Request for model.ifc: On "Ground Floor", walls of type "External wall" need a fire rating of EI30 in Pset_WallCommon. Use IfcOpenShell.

First a look at what the model holds.

```python
import ifcopenshell
import ifcopenshell.util.element

model = ifcopenshell.open("model.ifc")
print(model.schema)
storey = next(s for s in model.by_type("IfcBuildingStorey") if s.Name == "Ground Floor")
walls = [e for e in ifcopenshell.util.element.get_decomposition(storey) if e.is_a("IfcWall")]
seen = {}
for e in walls:
    element_type = ifcopenshell.util.element.get_type(e)
    key = (element_type.Name if element_type != e and element_type else None, ifcopenshell.util.element.get_pset(e, "Pset_WallCommon", "FireRating"))
    seen[key] = seen.get(key, 0) + 1
for (name, value), count in sorted(seen.items(), key=str):
    print(count, "x", name, "|", value)
```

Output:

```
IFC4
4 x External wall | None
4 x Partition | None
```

```python
import ifcopenshell
import ifcopenshell.api.pset
import ifcopenshell.util.element

model = ifcopenshell.open("model.ifc")

storey = next(s for s in model.by_type("IfcBuildingStorey") if s.Name == "Ground Floor")
walls = [e for e in ifcopenshell.util.element.get_decomposition(storey) if e.is_a("IfcWall")]

count = 0
for e in walls:
    element_type = ifcopenshell.util.element.get_type(e)
    if element_type in (None, e) or element_type.Name != "External wall":
        continue
    # add_pset returns the element's existing set when there is one.
    pset = ifcopenshell.api.pset.add_pset(model, product=e, name="Pset_WallCommon")
    ifcopenshell.api.pset.edit_pset(model, pset=pset, properties={"FireRating": "EI30"})
    count += 1

print(count, "walls updated")

model.write("model_edited.ifc")
```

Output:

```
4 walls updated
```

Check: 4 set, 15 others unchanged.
